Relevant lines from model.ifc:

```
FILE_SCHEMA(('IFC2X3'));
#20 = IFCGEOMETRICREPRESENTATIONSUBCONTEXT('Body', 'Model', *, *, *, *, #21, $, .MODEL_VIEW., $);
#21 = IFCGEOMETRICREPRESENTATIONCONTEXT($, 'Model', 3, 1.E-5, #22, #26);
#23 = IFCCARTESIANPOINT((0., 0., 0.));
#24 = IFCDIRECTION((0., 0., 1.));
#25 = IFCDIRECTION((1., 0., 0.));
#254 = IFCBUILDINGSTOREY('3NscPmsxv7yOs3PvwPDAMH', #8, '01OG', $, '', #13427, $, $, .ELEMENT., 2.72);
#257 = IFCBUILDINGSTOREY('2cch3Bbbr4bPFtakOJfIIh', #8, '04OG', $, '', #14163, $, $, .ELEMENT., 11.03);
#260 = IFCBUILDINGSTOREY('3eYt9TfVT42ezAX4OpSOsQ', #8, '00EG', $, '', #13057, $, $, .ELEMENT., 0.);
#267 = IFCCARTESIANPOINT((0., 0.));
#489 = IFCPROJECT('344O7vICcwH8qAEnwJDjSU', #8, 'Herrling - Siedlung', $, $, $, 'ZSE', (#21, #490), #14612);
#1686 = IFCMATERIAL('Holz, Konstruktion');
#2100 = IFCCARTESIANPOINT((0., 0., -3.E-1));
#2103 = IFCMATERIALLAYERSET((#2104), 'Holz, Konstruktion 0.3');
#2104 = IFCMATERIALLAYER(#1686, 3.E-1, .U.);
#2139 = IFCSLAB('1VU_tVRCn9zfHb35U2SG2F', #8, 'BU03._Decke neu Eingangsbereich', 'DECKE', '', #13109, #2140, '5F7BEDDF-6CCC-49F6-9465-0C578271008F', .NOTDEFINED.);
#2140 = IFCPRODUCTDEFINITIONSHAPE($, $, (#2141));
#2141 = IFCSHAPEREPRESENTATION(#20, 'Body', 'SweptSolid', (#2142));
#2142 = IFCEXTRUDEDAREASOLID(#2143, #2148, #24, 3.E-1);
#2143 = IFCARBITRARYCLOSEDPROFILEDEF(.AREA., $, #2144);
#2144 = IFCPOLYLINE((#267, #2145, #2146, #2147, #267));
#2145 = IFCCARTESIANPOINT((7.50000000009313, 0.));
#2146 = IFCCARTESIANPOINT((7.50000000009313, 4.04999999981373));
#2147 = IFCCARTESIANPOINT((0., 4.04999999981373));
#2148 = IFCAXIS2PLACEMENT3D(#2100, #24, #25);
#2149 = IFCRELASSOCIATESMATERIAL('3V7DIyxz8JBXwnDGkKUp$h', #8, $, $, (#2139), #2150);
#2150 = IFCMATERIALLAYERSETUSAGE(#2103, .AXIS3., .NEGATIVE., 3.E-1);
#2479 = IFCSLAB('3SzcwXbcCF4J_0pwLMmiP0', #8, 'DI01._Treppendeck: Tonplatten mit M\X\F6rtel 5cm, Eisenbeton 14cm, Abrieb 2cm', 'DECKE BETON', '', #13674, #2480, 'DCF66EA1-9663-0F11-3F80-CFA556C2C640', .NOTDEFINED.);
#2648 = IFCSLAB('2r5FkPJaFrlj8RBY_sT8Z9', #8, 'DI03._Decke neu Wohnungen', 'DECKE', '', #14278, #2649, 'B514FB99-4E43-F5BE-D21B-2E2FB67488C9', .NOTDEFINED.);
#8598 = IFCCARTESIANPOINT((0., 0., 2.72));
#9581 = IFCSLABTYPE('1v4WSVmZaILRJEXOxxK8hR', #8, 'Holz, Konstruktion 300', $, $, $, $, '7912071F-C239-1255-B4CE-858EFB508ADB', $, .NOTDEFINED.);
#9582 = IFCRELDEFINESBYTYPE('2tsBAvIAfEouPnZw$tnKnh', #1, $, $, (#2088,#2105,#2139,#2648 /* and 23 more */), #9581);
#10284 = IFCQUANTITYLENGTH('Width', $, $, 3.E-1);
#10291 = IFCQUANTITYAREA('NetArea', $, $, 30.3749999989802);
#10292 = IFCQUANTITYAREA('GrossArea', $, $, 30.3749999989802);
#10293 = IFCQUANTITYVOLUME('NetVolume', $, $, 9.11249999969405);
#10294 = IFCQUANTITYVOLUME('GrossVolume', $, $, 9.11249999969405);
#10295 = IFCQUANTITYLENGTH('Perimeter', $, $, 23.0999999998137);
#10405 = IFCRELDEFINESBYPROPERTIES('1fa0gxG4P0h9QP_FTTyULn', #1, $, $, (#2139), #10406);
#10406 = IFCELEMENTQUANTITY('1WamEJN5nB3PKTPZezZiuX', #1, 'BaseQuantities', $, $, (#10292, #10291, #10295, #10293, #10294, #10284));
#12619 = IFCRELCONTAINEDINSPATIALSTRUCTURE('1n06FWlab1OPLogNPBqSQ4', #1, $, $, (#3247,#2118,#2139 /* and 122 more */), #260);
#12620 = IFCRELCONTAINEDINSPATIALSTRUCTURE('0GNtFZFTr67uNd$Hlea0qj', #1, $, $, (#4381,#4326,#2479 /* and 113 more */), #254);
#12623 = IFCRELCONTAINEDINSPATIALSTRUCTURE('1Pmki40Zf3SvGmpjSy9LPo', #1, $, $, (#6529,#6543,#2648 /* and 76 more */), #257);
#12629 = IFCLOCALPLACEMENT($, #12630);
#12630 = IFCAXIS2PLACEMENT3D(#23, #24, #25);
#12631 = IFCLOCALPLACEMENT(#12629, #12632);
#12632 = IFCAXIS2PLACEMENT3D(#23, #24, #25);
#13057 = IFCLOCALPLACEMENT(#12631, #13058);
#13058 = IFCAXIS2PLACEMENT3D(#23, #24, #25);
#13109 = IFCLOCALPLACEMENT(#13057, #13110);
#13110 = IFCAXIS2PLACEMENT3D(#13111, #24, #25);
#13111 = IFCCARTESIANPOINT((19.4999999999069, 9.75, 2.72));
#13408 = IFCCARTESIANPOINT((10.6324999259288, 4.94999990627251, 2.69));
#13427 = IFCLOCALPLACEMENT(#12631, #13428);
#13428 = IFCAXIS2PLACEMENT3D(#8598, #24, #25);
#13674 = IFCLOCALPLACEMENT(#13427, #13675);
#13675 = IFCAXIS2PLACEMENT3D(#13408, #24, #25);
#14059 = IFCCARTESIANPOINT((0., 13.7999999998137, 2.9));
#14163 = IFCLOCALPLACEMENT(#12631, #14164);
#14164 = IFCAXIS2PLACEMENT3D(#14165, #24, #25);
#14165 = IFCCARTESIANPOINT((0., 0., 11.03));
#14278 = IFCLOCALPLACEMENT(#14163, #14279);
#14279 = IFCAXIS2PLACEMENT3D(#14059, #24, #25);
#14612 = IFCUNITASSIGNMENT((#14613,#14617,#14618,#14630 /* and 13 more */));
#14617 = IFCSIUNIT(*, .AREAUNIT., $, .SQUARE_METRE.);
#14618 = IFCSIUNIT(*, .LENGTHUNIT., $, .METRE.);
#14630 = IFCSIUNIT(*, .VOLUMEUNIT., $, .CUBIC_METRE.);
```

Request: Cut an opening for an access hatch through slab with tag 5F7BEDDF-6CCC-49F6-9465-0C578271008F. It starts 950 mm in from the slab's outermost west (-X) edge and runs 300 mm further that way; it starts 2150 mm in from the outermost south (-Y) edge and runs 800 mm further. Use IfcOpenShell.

```python
import numpy as np
import ifcopenshell
import ifcopenshell.api.feature
import ifcopenshell.api.geometry
import ifcopenshell.api.pset
import ifcopenshell.api.root
import ifcopenshell.geom
import ifcopenshell.util.element
import ifcopenshell.util.placement
import ifcopenshell.util.representation
import ifcopenshell.util.shape
import ifcopenshell.util.unit

model = ifcopenshell.open("model.ifc")
unit_scale = ifcopenshell.util.unit.calculate_unit_scale(model)
area_scale = ifcopenshell.util.unit.calculate_unit_scale(model, "AREAUNIT")
volume_scale = ifcopenshell.util.unit.calculate_unit_scale(model, "VOLUMEUNIT")
settings = ifcopenshell.geom.settings()


def volume(element):
    """Net volume in cubic metres, openings subtracted."""
    shape = ifcopenshell.geom.create_shape(settings, element)
    return ifcopenshell.util.shape.get_volume(shape.geometry)


slab = model.by_guid("1VU_tVRCn9zfHb35U2SG2F")
before = volume(slab)

# Extent in the slab's own axes, in metres. The edges named are its -X and -Y sides.
slab_shape = ifcopenshell.geom.create_shape(settings, slab)
vertices = ifcopenshell.util.shape.get_vertices(slab_shape.geometry)
x_min, y_min, bottom = vertices.min(axis=0)
top = vertices[:, 2].max()

opening = ifcopenshell.api.root.create_entity(model, ifc_class="IfcOpeningElement", name="Access hatch opening")
context = ifcopenshell.util.representation.get_context(model, "Model", "Body", "MODEL_VIEW")
width, depth = 0.3, 0.8
outline = [(0.0, 0.0), (width, 0.0), (width, depth), (0.0, depth), (0.0, 0.0)]
# Overshoot both faces by 50 mm so the cut is clean.
shape = ifcopenshell.api.geometry.add_slab_representation(
    model, context=context, depth=top - bottom + 0.1, polyline=outline
)
ifcopenshell.api.geometry.assign_representation(model, product=opening, representation=shape)

matrix = ifcopenshell.util.placement.get_local_placement(slab.ObjectPlacement)
matrix[:, 3] = matrix @ np.append(np.array([x_min + 0.95, y_min + 2.15, bottom - 0.05]) / unit_scale, 1.0)
ifcopenshell.api.geometry.edit_object_placement(model, product=opening, matrix=matrix, is_si=False)
ifcopenshell.api.feature.add_feature(model, feature=opening, element=slab)

after = volume(slab)

# Update the slab's stored quantities.
qto = model.by_id(ifcopenshell.util.element.get_pset(slab, "BaseQuantities", should_inherit=False)["id"])
ifcopenshell.api.pset.edit_qto(model, qto=qto, properties={
    "NetArea": after / (top - bottom) / area_scale,
    "NetVolume": after / volume_scale,
})

print(f"slab volume {before:.3f} -> {after:.3f} m3")

model.write("model_updated.ifc")
```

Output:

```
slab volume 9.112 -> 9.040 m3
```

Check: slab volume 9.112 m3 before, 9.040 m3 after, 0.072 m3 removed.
